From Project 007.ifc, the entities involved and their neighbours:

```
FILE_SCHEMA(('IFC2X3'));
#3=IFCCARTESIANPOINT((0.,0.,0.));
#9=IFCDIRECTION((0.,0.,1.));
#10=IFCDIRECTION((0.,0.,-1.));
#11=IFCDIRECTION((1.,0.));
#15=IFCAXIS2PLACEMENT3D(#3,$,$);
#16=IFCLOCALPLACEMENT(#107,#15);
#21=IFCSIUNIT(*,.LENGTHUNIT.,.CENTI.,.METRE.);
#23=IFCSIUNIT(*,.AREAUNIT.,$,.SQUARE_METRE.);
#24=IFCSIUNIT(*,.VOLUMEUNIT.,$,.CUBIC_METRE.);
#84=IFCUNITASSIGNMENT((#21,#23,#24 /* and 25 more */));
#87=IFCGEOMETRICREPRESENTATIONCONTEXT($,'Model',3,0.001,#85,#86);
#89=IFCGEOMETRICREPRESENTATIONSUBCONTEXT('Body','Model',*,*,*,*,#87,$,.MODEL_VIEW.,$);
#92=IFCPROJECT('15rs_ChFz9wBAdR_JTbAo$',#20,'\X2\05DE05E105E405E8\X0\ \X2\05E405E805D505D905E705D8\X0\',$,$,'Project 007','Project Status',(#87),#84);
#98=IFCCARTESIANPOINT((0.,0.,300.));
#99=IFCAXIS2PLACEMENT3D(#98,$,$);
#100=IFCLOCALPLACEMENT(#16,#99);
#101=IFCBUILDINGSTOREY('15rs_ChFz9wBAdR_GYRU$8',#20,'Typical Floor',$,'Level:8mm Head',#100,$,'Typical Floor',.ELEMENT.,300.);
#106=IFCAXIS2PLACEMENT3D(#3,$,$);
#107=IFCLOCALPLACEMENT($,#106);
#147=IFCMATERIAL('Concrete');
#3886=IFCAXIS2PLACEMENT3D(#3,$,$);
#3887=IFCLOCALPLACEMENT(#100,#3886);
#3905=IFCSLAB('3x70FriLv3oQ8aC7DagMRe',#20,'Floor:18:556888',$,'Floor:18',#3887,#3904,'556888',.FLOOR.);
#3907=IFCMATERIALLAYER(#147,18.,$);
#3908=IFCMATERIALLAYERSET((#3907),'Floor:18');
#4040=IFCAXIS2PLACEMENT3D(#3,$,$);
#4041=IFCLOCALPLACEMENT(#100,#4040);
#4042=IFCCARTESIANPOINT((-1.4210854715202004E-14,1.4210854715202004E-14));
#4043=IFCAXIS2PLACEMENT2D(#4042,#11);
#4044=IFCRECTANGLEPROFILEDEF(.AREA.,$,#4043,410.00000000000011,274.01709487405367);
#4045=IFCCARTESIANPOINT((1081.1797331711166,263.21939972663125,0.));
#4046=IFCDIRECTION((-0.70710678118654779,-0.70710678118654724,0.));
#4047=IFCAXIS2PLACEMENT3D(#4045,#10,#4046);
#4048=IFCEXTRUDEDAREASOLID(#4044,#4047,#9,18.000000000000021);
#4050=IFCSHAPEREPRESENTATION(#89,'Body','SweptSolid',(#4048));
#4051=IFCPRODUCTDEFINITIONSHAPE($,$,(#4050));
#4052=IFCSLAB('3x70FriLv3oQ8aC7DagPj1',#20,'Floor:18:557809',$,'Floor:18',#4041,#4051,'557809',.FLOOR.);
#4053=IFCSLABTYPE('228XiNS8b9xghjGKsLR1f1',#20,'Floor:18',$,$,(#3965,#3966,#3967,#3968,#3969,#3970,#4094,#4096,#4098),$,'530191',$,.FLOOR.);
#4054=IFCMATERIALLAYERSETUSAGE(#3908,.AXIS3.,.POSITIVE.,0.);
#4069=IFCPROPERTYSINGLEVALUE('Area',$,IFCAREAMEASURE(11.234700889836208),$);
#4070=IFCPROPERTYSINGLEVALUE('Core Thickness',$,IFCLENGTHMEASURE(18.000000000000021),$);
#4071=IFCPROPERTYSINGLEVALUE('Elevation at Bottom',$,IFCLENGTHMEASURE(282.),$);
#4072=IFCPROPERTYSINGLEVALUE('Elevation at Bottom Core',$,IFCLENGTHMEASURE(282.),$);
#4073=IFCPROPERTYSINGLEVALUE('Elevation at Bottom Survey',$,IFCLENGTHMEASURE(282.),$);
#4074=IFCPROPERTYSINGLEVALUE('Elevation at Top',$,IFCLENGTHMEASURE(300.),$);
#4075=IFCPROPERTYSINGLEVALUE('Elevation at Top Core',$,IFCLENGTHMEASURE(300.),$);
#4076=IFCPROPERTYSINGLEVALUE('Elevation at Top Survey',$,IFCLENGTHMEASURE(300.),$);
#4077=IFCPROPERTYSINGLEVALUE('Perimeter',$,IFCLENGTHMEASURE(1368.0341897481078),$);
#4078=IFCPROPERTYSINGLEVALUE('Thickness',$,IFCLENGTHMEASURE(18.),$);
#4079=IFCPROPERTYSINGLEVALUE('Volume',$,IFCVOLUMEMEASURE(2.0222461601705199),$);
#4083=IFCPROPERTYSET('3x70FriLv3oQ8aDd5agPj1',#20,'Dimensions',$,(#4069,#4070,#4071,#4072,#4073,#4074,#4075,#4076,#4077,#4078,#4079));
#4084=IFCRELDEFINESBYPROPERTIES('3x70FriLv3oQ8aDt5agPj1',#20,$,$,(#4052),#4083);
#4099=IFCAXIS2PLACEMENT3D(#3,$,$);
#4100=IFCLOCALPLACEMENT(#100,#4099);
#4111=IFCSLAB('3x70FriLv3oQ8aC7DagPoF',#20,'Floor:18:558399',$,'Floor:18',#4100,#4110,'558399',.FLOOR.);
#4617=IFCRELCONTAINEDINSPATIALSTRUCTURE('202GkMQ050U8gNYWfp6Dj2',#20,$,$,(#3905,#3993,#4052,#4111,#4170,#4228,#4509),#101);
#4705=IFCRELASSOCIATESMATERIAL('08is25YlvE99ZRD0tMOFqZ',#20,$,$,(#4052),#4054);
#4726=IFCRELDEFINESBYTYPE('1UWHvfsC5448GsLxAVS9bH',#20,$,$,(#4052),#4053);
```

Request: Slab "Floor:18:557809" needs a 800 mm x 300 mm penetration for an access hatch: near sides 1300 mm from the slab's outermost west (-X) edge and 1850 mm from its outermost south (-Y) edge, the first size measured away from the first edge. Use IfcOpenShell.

```python
import numpy as np
import ifcopenshell
import ifcopenshell.api.feature
import ifcopenshell.api.geometry
import ifcopenshell.api.pset
import ifcopenshell.api.root
import ifcopenshell.geom
import ifcopenshell.util.element
import ifcopenshell.util.placement
import ifcopenshell.util.representation
import ifcopenshell.util.shape
import ifcopenshell.util.unit

model = ifcopenshell.open("Project 007.ifc")
unit_scale = ifcopenshell.util.unit.calculate_unit_scale(model)
area_scale = ifcopenshell.util.unit.calculate_unit_scale(model, "AREAUNIT")
volume_scale = ifcopenshell.util.unit.calculate_unit_scale(model, "VOLUMEUNIT")
settings = ifcopenshell.geom.settings()


def volume(element):
    """Net volume in cubic metres, openings subtracted."""
    shape = ifcopenshell.geom.create_shape(settings, element)
    return ifcopenshell.util.shape.get_volume(shape.geometry)


slab = model.by_guid("3x70FriLv3oQ8aC7DagPj1")
before = volume(slab)

# Extent in the slab's own axes, in metres. The edges named are its -X and -Y sides.
slab_shape = ifcopenshell.geom.create_shape(settings, slab)
vertices = ifcopenshell.util.shape.get_vertices(slab_shape.geometry)
x_min, y_min, bottom = vertices.min(axis=0)
top = vertices[:, 2].max()

opening = ifcopenshell.api.root.create_entity(model, ifc_class="IfcOpeningElement", name="Access hatch opening")
context = ifcopenshell.util.representation.get_context(model, "Model", "Body", "MODEL_VIEW")
width, depth = 0.8, 0.3
outline = [(0.0, 0.0), (width, 0.0), (width, depth), (0.0, depth), (0.0, 0.0)]
# Overshoot both faces by 50 mm so the cut is clean.
shape = ifcopenshell.api.geometry.add_slab_representation(
    model, context=context, depth=top - bottom + 0.1, polyline=outline
)
ifcopenshell.api.geometry.assign_representation(model, product=opening, representation=shape)

matrix = ifcopenshell.util.placement.get_local_placement(slab.ObjectPlacement)
matrix[:, 3] = matrix @ np.append(np.array([x_min + 1.3, y_min + 1.85, bottom - 0.05]) / unit_scale, 1.0)
ifcopenshell.api.geometry.edit_object_placement(model, product=opening, matrix=matrix, is_si=False)
ifcopenshell.api.feature.add_feature(model, feature=opening, element=slab)

after = volume(slab)

# Update the slab's stored quantities.
pset = model.by_id(ifcopenshell.util.element.get_pset(slab, "Dimensions", should_inherit=False)["id"])
ifcopenshell.api.pset.edit_pset(model, pset=pset, properties={
    "Area": model.create_entity("IfcAreaMeasure", after / (top - bottom) / area_scale),
    "Volume": model.create_entity("IfcVolumeMeasure", after / volume_scale),
})

print(f"slab volume {before:.3f} -> {after:.3f} m3")

model.write("Project 007-out.ifc")
```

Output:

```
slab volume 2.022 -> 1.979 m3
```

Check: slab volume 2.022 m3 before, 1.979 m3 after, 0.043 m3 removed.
